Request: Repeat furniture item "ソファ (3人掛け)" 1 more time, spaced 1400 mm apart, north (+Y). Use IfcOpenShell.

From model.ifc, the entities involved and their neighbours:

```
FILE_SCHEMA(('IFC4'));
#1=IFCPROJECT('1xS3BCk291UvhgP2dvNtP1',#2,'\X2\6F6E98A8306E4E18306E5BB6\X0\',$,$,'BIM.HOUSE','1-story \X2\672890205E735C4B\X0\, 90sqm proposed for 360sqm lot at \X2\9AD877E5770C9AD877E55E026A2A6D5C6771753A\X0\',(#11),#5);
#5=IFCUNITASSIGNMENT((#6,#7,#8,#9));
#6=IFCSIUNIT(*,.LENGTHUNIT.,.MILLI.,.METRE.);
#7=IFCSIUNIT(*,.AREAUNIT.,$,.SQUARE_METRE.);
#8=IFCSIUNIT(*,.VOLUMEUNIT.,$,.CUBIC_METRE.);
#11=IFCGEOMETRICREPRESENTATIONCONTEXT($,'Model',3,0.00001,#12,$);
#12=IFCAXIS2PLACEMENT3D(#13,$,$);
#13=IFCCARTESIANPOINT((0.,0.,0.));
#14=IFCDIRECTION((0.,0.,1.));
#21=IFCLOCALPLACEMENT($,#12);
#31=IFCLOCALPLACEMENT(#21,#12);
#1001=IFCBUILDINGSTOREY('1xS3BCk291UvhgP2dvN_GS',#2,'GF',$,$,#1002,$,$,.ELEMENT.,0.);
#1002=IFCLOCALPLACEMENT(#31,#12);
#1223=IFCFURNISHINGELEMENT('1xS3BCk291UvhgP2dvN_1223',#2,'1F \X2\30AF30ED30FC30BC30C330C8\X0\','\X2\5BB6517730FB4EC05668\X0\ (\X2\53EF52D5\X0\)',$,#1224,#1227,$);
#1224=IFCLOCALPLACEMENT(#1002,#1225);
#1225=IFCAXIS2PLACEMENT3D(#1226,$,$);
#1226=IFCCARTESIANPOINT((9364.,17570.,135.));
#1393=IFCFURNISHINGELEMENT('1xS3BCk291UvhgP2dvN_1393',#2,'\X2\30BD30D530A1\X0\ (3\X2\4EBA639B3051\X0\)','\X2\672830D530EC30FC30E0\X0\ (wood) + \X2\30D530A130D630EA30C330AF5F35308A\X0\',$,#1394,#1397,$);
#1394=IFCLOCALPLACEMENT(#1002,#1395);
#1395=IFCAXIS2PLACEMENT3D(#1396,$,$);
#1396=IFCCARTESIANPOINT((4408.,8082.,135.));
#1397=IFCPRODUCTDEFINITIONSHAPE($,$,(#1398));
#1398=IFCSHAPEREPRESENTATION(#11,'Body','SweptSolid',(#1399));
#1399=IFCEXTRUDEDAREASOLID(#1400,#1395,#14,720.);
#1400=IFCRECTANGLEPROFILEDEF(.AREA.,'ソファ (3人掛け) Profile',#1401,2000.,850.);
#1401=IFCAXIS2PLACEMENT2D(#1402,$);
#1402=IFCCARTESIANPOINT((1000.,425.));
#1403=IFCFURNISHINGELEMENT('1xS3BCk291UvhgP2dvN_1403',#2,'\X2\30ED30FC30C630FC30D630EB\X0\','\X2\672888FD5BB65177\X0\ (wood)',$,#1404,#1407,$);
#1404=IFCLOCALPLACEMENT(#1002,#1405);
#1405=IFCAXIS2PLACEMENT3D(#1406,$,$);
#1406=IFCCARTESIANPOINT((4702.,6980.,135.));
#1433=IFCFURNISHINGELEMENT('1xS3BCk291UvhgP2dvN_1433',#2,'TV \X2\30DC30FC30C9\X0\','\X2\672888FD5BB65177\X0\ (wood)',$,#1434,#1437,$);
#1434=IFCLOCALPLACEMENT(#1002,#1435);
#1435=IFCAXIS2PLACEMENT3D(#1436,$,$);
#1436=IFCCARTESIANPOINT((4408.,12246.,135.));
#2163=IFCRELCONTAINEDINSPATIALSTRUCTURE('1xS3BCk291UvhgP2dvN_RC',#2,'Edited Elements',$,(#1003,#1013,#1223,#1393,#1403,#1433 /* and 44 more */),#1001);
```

```python
import numpy as np
import ifcopenshell
import ifcopenshell.api.geometry
import ifcopenshell.api.root
import ifcopenshell.util.element
import ifcopenshell.util.placement
import ifcopenshell.util.unit

model = ifcopenshell.open("model.ifc")
unit_scale = ifcopenshell.util.unit.calculate_unit_scale(model)


def reuse_history(source, copy):
    """copy_class also copies each property set's owner history, people and application; keep the originals."""
    for rel in copy.IsDefinedBy:
        if rel.is_a("IfcRelDefinesByProperties") and (history := rel.RelatingPropertyDefinition.OwnerHistory):
            rel.RelatingPropertyDefinition.OwnerHistory = source.OwnerHistory
            ifcopenshell.util.element.remove_deep2(model, history)


source = model.by_id(1393)
base = ifcopenshell.util.placement.get_local_placement(source.ObjectPlacement)
step = np.array([0.0, 1.0, 0.0]) * 1.4 / unit_scale

for i in range(1, 2):
    copy = ifcopenshell.api.root.copy_class(model, product=source)
    copy.Representation = ifcopenshell.util.element.copy_deep(
        model, source.Representation, exclude=["IfcGeometricRepresentationContext", "IfcRepresentationMap"]
    )
    reuse_history(source, copy)
    matrix = base.copy()
    matrix[:3, 3] += i * step
    print("added at", matrix[:3, 3].round(3) + 0.0)
    ifcopenshell.api.geometry.edit_object_placement(model, product=copy, matrix=matrix, is_si=False)

model.write("model_edited.ifc")
```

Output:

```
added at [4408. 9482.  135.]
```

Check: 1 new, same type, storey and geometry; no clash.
